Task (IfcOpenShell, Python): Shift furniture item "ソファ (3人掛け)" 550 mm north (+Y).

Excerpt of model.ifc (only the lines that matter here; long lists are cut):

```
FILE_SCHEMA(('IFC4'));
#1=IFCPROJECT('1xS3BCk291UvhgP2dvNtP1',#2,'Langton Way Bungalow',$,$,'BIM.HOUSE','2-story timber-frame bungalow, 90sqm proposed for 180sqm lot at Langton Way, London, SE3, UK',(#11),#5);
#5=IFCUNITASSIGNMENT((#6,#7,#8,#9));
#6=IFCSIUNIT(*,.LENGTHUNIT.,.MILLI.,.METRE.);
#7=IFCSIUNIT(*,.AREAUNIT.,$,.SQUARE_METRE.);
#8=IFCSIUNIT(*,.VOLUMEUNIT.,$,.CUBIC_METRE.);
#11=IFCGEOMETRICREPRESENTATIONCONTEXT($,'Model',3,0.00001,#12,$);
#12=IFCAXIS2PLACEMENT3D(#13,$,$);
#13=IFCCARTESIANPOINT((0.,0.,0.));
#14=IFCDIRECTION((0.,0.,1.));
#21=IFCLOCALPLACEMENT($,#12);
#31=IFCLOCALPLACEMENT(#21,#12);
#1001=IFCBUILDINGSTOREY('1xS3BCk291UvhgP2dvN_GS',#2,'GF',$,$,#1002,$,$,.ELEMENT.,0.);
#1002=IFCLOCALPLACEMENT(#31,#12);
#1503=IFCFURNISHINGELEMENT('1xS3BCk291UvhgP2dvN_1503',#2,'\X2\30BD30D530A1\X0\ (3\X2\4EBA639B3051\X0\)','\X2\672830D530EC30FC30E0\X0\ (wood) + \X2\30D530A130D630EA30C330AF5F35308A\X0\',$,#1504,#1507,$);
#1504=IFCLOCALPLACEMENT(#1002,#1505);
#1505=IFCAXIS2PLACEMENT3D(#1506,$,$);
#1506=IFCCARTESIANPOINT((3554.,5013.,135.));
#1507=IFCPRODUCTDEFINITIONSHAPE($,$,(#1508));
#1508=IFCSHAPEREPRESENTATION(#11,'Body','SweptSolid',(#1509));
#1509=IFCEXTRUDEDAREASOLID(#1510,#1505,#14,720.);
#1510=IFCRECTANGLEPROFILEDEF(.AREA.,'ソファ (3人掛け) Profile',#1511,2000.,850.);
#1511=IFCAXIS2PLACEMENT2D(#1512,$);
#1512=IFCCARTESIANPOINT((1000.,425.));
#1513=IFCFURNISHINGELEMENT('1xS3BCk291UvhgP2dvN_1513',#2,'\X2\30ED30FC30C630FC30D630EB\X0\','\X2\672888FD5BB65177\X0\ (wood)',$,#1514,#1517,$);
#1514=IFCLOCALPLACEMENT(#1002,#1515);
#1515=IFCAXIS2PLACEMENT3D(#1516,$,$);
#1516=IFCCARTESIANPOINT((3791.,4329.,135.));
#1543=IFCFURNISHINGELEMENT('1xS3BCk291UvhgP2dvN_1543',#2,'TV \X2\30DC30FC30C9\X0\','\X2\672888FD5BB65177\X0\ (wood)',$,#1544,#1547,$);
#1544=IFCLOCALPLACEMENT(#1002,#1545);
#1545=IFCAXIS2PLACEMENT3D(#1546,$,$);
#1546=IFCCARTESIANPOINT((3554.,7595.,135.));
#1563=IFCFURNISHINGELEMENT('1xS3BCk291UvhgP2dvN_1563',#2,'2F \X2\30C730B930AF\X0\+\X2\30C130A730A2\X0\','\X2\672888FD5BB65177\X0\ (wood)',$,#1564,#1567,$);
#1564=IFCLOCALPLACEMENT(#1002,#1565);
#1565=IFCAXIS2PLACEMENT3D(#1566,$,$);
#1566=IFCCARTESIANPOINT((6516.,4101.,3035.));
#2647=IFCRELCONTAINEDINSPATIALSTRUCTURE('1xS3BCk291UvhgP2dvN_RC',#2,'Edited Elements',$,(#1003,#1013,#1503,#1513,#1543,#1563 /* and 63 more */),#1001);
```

```python
import ifcopenshell
import ifcopenshell.api.geometry
import ifcopenshell.util.placement
import ifcopenshell.util.unit

model = ifcopenshell.open("model.ifc")
unit_scale = ifcopenshell.util.unit.calculate_unit_scale(model)

item = model.by_guid("1xS3BCk291UvhgP2dvN_1503")
matrix = ifcopenshell.util.placement.get_local_placement(item.ObjectPlacement)
matrix[1, 3] += 0.55 / unit_scale
ifcopenshell.api.geometry.edit_object_placement(model, product=item, matrix=matrix, is_si=False)

print(ifcopenshell.util.placement.get_local_placement(item.ObjectPlacement).round(3) + 0.0)

model.write("model-out.ifc")
```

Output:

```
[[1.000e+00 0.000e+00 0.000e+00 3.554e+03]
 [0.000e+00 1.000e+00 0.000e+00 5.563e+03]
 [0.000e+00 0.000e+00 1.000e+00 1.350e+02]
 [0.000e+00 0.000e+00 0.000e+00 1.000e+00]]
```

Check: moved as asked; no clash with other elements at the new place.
